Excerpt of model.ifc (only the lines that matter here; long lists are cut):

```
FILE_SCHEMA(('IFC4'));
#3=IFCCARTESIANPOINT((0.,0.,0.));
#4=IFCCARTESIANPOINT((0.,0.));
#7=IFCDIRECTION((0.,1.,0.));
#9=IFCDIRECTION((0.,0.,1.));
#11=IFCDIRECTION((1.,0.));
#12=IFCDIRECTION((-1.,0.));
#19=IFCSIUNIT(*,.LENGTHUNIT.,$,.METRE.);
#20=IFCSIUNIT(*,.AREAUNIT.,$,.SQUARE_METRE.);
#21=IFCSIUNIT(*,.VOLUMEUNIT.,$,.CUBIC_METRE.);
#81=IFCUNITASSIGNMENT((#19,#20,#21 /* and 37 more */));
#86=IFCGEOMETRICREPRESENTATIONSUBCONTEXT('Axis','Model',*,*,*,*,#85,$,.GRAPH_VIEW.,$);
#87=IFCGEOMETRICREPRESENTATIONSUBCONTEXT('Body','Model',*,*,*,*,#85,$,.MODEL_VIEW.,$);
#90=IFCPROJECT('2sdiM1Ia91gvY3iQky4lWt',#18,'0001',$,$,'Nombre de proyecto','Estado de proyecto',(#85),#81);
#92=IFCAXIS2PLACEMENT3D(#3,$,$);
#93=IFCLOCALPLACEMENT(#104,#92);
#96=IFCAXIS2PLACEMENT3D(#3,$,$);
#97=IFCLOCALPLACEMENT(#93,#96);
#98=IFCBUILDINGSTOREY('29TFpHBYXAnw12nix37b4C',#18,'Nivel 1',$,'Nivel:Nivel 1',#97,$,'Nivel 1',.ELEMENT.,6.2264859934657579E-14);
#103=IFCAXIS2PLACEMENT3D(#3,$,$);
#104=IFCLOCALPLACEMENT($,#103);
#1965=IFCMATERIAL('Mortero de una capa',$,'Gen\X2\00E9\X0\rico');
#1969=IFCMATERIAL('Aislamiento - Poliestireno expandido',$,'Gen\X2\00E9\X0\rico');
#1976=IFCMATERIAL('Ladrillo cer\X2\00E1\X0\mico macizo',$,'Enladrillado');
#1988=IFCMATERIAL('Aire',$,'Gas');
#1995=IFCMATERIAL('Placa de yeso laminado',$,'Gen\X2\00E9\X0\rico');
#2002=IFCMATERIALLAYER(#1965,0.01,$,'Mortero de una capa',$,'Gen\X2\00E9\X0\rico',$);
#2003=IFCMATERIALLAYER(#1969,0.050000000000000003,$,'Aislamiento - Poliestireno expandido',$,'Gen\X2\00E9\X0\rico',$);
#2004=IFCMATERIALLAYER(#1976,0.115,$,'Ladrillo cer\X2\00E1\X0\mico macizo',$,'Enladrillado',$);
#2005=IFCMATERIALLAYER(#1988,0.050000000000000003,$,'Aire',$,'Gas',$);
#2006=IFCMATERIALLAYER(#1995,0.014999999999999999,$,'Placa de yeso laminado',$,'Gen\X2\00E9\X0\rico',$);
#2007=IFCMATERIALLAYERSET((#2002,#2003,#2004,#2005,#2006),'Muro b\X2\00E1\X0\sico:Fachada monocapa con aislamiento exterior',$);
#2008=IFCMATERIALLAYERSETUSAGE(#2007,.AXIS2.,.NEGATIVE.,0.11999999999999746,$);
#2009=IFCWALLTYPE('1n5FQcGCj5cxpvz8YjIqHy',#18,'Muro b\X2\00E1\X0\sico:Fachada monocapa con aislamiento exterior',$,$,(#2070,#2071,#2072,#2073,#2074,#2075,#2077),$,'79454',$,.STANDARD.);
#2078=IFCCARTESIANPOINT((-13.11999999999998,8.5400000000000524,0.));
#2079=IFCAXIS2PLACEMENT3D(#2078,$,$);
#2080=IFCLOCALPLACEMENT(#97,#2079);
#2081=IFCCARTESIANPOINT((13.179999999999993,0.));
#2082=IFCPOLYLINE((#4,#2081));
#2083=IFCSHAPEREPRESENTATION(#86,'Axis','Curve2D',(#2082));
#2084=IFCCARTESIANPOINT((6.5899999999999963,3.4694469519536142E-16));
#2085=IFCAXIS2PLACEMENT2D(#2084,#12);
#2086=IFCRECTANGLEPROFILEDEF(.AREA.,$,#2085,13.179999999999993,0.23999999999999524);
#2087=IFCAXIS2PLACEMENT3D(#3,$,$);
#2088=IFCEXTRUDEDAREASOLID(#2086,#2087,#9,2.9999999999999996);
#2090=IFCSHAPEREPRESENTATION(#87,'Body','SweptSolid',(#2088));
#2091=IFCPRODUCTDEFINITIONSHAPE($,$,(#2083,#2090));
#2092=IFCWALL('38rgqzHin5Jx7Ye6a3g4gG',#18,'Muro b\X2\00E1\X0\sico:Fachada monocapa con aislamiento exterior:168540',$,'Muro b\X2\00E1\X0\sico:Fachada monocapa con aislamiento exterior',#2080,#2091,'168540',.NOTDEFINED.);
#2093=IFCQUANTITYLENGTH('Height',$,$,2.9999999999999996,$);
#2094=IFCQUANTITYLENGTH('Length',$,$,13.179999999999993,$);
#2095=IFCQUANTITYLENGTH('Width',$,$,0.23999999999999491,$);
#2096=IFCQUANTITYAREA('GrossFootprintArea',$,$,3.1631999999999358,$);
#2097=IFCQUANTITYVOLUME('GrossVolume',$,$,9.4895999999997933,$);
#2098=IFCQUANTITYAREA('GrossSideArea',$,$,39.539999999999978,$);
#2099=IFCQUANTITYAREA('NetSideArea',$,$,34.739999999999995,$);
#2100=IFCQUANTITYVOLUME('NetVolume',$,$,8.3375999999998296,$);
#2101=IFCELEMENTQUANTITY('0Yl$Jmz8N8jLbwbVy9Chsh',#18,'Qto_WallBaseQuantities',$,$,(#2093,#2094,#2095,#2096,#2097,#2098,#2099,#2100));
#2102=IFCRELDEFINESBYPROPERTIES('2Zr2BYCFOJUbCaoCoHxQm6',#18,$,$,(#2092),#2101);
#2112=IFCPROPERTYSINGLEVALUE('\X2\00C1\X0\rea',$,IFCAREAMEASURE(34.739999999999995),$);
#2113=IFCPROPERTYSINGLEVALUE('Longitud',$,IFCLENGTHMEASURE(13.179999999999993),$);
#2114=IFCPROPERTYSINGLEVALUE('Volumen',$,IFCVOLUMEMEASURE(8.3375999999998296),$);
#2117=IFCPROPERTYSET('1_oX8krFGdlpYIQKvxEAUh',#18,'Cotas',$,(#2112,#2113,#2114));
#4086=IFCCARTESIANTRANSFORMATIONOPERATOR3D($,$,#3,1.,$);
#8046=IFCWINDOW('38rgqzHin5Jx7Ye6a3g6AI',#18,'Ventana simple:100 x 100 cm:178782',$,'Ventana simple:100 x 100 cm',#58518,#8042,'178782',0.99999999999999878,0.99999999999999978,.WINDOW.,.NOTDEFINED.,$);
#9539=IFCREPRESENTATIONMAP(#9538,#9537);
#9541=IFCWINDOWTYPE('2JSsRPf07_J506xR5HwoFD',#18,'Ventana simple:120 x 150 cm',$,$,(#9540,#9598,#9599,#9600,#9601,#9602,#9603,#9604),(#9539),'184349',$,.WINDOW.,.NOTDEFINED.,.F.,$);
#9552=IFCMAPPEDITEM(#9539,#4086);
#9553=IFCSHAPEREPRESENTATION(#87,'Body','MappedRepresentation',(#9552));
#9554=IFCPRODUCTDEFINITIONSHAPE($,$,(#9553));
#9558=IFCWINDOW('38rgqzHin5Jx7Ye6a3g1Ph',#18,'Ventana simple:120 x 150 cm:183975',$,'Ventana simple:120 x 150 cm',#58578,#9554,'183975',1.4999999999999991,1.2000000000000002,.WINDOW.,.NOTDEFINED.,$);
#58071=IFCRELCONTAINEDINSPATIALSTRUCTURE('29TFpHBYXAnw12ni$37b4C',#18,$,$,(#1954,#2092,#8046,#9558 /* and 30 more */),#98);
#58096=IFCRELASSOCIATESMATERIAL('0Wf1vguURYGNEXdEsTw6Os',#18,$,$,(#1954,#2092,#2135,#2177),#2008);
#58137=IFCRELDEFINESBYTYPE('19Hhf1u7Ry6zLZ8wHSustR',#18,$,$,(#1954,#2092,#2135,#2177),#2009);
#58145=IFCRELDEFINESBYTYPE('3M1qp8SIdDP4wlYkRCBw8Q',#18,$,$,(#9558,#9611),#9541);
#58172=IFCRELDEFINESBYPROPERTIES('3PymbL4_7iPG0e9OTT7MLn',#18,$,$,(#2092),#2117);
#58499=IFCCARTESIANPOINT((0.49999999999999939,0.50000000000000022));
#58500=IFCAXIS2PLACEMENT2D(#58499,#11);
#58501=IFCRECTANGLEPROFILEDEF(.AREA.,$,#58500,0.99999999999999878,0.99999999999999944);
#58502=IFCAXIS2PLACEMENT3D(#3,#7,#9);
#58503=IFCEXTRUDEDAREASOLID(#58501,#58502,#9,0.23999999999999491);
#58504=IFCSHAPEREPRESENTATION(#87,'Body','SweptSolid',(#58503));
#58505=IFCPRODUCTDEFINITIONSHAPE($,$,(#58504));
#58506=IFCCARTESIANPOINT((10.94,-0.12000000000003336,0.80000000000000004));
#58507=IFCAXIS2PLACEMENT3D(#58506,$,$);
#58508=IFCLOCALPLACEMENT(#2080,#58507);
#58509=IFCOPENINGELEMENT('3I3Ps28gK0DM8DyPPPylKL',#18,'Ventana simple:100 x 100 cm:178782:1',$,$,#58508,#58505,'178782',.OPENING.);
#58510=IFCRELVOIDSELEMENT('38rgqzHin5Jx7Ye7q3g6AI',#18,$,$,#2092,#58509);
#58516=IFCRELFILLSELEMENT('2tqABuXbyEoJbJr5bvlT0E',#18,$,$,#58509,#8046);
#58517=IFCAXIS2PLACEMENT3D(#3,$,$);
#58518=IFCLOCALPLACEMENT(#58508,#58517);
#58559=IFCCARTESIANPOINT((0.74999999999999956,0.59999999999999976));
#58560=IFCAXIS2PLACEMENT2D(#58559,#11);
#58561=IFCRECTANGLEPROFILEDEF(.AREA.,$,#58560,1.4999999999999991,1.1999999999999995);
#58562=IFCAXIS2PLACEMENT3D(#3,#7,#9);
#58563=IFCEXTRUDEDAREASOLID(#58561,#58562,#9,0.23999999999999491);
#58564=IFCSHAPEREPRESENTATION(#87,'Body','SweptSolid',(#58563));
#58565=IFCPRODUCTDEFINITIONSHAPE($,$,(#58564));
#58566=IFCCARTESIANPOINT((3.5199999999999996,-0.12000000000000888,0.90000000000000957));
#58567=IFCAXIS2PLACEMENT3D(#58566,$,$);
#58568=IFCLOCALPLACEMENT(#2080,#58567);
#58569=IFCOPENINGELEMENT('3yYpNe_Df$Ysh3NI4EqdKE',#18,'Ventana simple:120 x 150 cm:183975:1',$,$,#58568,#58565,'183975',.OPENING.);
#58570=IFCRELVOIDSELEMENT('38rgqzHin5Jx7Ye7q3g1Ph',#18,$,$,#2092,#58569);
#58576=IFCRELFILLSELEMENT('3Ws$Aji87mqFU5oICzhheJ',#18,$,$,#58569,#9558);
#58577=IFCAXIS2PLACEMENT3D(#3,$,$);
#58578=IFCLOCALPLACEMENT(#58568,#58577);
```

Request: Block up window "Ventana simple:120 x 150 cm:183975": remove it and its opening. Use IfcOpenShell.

```python
import ifcopenshell
import ifcopenshell.api.feature
import ifcopenshell.api.pset
import ifcopenshell.api.root
import ifcopenshell.geom
import ifcopenshell.util.element
import ifcopenshell.util.shape
import ifcopenshell.util.unit

model = ifcopenshell.open("model.ifc")
area_scale = ifcopenshell.util.unit.calculate_unit_scale(model, "AREAUNIT")
volume_scale = ifcopenshell.util.unit.calculate_unit_scale(model, "VOLUMEUNIT")
settings = ifcopenshell.geom.settings()


def volume(element):
    """Net volume in cubic metres, openings subtracted."""
    shape = ifcopenshell.geom.create_shape(settings, element)
    return ifcopenshell.util.shape.get_volume(shape.geometry)


window = model.by_guid("38rgqzHin5Jx7Ye6a3g1Ph")
opening = window.FillsVoids[0].RelatingOpeningElement
wall = opening.VoidsElements[0].RelatingBuildingElement
before = volume(wall)

ifcopenshell.api.root.remove_product(model, product=window)
ifcopenshell.api.feature.remove_feature(model, feature=opening)

after = volume(wall)
thickness = 0.24  # wall thickness in metres

# Update the wall's stored quantities.
qto = model.by_id(ifcopenshell.util.element.get_pset(wall, "Qto_WallBaseQuantities", should_inherit=False)["id"])
ifcopenshell.api.pset.edit_qto(model, qto=qto, properties={
    "NetSideArea": after / thickness / area_scale,
    "NetVolume": after / volume_scale,
})
pset = model.by_id(ifcopenshell.util.element.get_pset(wall, "Cotas", should_inherit=False)["id"])
ifcopenshell.api.pset.edit_pset(model, pset=pset, properties={
    "Área": model.create_entity("IfcAreaMeasure", after / thickness / area_scale),
    "Volumen": model.create_entity("IfcVolumeMeasure", after / volume_scale),
})

print(f"wall volume {before:.3f} -> {after:.3f} m3")

model.write("model_v2.ifc")
```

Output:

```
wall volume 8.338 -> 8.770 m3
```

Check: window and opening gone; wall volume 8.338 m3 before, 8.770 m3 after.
